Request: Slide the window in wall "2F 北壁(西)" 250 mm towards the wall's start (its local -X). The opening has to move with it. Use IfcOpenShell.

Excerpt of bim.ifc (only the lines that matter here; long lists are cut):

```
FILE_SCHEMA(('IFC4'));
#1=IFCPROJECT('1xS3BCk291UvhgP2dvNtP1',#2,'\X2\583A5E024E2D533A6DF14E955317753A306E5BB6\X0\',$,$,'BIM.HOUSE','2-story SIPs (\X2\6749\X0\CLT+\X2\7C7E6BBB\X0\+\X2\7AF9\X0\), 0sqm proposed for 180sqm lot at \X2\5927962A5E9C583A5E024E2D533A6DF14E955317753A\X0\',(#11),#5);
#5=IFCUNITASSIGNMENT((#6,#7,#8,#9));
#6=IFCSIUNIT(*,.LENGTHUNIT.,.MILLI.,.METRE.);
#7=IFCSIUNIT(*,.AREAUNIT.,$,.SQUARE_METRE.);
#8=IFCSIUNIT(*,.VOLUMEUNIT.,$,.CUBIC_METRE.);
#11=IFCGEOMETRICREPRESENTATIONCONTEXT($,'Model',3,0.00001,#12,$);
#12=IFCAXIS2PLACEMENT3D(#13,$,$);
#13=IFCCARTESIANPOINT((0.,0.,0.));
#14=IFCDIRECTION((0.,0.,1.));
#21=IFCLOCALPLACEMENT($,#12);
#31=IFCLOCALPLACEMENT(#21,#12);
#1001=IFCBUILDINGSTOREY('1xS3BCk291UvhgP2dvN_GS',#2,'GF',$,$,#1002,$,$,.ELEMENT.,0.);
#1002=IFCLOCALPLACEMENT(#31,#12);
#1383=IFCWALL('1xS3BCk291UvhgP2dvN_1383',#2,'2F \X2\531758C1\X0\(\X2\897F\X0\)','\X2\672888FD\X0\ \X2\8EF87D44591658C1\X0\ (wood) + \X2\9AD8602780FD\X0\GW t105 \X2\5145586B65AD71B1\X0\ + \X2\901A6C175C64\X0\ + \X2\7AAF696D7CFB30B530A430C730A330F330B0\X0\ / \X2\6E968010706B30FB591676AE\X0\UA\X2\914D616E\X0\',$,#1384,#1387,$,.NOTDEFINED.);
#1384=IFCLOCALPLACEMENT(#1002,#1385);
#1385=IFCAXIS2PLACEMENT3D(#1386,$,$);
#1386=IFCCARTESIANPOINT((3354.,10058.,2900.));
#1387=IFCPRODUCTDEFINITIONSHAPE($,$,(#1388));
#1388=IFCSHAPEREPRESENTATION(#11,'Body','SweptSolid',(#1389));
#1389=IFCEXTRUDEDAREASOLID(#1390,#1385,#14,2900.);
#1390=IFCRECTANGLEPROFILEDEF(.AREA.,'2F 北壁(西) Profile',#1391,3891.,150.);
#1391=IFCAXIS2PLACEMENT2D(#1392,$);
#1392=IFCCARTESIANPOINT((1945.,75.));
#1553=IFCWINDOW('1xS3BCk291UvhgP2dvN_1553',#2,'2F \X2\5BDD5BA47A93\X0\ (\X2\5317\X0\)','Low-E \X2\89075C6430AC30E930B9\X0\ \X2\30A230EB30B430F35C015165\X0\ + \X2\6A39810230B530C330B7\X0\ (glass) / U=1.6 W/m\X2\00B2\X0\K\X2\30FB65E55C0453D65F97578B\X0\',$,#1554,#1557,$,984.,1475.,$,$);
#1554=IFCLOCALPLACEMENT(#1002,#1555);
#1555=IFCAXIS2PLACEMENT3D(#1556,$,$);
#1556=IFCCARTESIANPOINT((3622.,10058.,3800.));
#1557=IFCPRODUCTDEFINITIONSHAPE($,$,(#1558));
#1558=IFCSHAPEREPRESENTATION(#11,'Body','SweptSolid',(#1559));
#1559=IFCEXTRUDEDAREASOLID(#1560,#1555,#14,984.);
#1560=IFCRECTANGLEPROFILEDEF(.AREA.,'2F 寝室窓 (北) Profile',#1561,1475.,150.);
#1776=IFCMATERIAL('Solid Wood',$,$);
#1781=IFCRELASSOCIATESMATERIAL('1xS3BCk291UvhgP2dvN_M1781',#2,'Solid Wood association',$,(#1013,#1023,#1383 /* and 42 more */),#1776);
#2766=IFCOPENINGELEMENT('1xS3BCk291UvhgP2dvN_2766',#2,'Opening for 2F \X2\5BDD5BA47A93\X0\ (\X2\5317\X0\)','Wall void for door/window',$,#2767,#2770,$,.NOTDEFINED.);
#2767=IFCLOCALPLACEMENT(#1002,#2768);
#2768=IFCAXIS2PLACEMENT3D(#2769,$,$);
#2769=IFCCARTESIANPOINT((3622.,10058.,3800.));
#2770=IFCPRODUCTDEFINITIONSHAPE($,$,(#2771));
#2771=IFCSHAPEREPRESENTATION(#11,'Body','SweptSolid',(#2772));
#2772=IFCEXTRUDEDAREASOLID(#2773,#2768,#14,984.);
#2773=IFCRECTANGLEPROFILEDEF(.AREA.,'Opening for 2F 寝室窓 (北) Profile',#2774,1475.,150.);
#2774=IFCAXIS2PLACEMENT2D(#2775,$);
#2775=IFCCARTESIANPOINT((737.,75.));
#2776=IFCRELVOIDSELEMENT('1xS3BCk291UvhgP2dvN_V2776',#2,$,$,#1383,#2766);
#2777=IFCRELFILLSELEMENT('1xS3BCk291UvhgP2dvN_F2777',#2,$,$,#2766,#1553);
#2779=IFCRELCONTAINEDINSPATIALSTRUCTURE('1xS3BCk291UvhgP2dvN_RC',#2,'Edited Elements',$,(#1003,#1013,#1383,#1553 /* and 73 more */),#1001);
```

```python
import ifcopenshell
import ifcopenshell.api.geometry
import ifcopenshell.util.placement

model = ifcopenshell.open("bim.ifc")

window = model.by_guid("1xS3BCk291UvhgP2dvN_1553")
opening = window.FillsVoids[0].RelatingOpeningElement
wall = opening.VoidsElements[0].RelatingBuildingElement

wall_matrix = ifcopenshell.util.placement.get_local_placement(wall.ObjectPlacement)
shift = wall_matrix[:3, 0] * -250.0
before = ifcopenshell.util.placement.get_local_placement(window.ObjectPlacement)[:3, 3].copy()

# The window is not placed relative to its opening, so move both.
for product in (opening, window):
    matrix = ifcopenshell.util.placement.get_local_placement(product.ObjectPlacement)
    matrix[:3, 3] += shift
    ifcopenshell.api.geometry.edit_object_placement(model, product=product, matrix=matrix, is_si=False)

after = ifcopenshell.util.placement.get_local_placement(window.ObjectPlacement)[:3, 3]
print("window moved by", (after - before).round(3) + 0.0)

model.write("bim_edited.ifc")
```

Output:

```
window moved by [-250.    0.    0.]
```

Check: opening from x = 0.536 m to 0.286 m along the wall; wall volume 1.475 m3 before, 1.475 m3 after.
